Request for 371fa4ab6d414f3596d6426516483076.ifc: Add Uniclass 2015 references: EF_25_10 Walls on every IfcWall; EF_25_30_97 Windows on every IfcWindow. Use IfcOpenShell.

First a look at what the model holds.

```python
import ifcopenshell

model = ifcopenshell.open("371fa4ab6d414f3596d6426516483076.ifc")
print(model.schema)
print("classifications:", [c.Name for c in model.by_type("IfcClassification")])
for ifc_class in ("IfcDoor", "IfcRoof", "IfcStair", "IfcWall", "IfcWindow"):
    print(ifc_class, len(model.by_type(ifc_class)))
```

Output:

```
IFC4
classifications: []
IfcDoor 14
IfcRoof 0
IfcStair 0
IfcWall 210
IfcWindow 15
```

```python
import ifcopenshell
import ifcopenshell.api.classification

model = ifcopenshell.open("371fa4ab6d414f3596d6426516483076.ifc")

system = ifcopenshell.api.classification.add_classification(model, classification="Uniclass 2015")

codes = {
    "IfcWall": ("EF_25_10", "Walls"),
    "IfcWindow": ("EF_25_30_97", "Windows"),
}
for ifc_class, (code, name) in codes.items():
    products = model.by_type(ifc_class)
    ifcopenshell.api.classification.add_reference(
        model, products=products, classification=system, identification=code, name=name
    )
    print(code, len(products))

model.write("371fa4ab6d414f3596d6426516483076_edited.ifc")
```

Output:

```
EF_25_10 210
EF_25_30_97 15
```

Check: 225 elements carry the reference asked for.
